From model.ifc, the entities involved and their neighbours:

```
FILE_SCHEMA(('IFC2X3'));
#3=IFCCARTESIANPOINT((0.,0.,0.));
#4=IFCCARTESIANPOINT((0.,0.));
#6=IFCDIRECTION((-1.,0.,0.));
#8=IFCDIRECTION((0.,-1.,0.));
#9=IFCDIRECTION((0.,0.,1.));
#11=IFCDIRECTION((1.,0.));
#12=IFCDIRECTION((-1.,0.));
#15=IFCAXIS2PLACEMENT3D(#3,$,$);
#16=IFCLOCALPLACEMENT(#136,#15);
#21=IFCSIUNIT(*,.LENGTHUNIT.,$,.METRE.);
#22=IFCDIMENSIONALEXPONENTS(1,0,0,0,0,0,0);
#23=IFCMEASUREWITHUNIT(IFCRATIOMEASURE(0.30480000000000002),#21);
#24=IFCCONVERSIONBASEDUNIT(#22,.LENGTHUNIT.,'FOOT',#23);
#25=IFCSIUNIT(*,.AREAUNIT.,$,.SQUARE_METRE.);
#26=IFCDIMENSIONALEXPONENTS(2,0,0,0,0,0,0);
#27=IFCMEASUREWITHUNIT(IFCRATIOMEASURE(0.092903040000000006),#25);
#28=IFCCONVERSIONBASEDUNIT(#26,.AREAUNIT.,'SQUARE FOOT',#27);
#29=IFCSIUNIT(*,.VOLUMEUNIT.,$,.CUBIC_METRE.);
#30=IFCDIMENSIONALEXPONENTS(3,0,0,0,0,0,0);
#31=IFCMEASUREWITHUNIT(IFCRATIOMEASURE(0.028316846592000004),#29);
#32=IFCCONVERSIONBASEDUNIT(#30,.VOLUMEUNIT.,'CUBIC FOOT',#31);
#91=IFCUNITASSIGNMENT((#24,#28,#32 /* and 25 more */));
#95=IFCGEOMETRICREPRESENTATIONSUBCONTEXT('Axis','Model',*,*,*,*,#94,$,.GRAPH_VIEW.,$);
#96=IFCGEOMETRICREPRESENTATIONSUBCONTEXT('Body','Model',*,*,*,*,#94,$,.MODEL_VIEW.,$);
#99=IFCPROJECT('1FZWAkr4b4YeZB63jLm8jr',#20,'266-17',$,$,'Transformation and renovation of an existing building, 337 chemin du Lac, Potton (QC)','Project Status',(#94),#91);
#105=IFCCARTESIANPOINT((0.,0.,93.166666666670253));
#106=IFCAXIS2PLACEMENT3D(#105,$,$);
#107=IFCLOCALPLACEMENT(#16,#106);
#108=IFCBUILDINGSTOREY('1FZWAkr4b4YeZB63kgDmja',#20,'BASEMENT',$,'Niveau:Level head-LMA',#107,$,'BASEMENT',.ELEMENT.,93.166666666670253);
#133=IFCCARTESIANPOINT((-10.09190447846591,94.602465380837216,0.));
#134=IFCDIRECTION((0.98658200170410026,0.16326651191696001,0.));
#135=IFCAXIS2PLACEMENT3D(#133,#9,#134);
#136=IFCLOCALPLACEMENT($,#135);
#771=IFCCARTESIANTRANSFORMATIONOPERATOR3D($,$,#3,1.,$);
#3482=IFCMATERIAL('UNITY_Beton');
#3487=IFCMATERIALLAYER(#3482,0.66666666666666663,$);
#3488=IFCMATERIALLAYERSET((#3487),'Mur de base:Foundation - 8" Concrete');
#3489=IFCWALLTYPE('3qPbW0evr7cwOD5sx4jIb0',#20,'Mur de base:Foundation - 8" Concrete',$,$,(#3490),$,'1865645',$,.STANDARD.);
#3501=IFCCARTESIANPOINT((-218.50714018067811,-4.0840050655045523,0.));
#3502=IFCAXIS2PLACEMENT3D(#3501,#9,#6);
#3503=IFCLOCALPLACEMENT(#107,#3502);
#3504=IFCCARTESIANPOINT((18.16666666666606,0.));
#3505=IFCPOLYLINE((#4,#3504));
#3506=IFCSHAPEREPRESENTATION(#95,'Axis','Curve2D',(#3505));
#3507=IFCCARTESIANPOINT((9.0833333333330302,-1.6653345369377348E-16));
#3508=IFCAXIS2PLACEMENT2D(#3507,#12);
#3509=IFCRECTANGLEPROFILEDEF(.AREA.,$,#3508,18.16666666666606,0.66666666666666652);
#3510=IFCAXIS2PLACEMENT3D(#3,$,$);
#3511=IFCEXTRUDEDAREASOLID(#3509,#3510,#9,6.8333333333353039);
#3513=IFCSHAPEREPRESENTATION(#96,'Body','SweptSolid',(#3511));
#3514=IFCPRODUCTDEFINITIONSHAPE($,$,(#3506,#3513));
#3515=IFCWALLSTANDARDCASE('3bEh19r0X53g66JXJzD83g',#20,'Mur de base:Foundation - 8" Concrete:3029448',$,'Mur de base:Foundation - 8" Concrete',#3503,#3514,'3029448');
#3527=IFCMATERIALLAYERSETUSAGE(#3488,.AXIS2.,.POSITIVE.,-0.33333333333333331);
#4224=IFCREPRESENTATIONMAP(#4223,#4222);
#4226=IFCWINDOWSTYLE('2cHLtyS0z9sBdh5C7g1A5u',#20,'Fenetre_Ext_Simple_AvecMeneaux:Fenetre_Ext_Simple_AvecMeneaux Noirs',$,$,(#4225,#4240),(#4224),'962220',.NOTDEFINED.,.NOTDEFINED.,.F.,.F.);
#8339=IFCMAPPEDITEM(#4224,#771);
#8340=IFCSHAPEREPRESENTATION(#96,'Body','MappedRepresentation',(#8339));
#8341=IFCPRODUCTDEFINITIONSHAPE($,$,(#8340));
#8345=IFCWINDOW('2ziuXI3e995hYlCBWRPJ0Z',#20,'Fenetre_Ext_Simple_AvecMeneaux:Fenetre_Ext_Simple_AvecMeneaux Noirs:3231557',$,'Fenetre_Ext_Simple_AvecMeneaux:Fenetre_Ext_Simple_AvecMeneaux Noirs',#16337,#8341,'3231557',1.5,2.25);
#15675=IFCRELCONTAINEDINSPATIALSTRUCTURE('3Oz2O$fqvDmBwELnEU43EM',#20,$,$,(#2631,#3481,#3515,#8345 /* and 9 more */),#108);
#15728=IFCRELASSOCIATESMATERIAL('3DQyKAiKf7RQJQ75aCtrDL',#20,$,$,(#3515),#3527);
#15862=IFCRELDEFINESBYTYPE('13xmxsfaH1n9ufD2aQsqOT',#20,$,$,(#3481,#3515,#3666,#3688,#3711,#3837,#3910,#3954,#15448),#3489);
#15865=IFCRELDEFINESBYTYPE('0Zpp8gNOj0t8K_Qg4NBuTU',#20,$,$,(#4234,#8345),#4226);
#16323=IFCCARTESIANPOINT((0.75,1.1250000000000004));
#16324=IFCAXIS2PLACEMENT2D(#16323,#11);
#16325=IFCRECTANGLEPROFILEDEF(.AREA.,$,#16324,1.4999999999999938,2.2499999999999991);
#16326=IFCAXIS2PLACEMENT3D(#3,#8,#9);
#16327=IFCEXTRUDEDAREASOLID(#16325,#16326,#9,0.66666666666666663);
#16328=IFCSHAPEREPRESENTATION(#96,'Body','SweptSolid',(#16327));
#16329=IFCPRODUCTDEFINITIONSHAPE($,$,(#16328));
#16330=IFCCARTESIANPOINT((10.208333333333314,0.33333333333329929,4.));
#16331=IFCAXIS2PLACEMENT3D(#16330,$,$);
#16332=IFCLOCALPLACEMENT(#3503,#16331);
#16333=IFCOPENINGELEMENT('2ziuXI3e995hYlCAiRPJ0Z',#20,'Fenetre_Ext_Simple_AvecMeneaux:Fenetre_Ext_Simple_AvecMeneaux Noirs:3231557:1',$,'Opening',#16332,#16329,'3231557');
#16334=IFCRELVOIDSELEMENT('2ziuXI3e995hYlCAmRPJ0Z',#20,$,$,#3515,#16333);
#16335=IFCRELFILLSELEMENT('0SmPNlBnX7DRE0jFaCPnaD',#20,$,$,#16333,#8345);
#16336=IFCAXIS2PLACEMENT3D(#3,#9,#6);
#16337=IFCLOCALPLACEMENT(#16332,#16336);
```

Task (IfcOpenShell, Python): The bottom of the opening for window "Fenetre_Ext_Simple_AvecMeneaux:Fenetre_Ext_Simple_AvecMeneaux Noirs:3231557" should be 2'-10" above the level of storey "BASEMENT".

```python
import numpy as np
import ifcopenshell
import ifcopenshell.api.geometry
import ifcopenshell.geom
import ifcopenshell.util.element
import ifcopenshell.util.placement
import ifcopenshell.util.shape
import ifcopenshell.util.unit

model = ifcopenshell.open("model.ifc")
unit_scale = ifcopenshell.util.unit.calculate_unit_scale(model)

window = model.by_guid("2ziuXI3e995hYlCBWRPJ0Z")
opening = window.FillsVoids[0].RelatingOpeningElement
storey = ifcopenshell.util.element.get_container(window, ifc_class="IfcBuildingStorey")
level = ifcopenshell.util.placement.get_local_placement(storey.ObjectPlacement)[2, 3]

# The opening's origin need not be at the sill, so measure its lowest point.
shape = ifcopenshell.geom.create_shape(ifcopenshell.geom.settings(), opening)
bottom = ifcopenshell.util.shape.get_shape_bottom_elevation(shape, shape.geometry) / unit_scale
dz = level + 34 * 0.0254 / unit_scale - bottom

shift = np.array([0.0, 0.0, dz])
# The window is placed relative to its opening, so it follows when the opening moves.
matrix = ifcopenshell.util.placement.get_local_placement(opening.ObjectPlacement)
matrix[:3, 3] += shift
ifcopenshell.api.geometry.edit_object_placement(
    model, product=opening, matrix=matrix, is_si=False, should_transform_children=True
)

print(f"moved by {dz * unit_scale:+.3f} m")

model.write("model_rev.ifc")
```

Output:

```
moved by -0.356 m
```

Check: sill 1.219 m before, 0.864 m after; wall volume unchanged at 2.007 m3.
